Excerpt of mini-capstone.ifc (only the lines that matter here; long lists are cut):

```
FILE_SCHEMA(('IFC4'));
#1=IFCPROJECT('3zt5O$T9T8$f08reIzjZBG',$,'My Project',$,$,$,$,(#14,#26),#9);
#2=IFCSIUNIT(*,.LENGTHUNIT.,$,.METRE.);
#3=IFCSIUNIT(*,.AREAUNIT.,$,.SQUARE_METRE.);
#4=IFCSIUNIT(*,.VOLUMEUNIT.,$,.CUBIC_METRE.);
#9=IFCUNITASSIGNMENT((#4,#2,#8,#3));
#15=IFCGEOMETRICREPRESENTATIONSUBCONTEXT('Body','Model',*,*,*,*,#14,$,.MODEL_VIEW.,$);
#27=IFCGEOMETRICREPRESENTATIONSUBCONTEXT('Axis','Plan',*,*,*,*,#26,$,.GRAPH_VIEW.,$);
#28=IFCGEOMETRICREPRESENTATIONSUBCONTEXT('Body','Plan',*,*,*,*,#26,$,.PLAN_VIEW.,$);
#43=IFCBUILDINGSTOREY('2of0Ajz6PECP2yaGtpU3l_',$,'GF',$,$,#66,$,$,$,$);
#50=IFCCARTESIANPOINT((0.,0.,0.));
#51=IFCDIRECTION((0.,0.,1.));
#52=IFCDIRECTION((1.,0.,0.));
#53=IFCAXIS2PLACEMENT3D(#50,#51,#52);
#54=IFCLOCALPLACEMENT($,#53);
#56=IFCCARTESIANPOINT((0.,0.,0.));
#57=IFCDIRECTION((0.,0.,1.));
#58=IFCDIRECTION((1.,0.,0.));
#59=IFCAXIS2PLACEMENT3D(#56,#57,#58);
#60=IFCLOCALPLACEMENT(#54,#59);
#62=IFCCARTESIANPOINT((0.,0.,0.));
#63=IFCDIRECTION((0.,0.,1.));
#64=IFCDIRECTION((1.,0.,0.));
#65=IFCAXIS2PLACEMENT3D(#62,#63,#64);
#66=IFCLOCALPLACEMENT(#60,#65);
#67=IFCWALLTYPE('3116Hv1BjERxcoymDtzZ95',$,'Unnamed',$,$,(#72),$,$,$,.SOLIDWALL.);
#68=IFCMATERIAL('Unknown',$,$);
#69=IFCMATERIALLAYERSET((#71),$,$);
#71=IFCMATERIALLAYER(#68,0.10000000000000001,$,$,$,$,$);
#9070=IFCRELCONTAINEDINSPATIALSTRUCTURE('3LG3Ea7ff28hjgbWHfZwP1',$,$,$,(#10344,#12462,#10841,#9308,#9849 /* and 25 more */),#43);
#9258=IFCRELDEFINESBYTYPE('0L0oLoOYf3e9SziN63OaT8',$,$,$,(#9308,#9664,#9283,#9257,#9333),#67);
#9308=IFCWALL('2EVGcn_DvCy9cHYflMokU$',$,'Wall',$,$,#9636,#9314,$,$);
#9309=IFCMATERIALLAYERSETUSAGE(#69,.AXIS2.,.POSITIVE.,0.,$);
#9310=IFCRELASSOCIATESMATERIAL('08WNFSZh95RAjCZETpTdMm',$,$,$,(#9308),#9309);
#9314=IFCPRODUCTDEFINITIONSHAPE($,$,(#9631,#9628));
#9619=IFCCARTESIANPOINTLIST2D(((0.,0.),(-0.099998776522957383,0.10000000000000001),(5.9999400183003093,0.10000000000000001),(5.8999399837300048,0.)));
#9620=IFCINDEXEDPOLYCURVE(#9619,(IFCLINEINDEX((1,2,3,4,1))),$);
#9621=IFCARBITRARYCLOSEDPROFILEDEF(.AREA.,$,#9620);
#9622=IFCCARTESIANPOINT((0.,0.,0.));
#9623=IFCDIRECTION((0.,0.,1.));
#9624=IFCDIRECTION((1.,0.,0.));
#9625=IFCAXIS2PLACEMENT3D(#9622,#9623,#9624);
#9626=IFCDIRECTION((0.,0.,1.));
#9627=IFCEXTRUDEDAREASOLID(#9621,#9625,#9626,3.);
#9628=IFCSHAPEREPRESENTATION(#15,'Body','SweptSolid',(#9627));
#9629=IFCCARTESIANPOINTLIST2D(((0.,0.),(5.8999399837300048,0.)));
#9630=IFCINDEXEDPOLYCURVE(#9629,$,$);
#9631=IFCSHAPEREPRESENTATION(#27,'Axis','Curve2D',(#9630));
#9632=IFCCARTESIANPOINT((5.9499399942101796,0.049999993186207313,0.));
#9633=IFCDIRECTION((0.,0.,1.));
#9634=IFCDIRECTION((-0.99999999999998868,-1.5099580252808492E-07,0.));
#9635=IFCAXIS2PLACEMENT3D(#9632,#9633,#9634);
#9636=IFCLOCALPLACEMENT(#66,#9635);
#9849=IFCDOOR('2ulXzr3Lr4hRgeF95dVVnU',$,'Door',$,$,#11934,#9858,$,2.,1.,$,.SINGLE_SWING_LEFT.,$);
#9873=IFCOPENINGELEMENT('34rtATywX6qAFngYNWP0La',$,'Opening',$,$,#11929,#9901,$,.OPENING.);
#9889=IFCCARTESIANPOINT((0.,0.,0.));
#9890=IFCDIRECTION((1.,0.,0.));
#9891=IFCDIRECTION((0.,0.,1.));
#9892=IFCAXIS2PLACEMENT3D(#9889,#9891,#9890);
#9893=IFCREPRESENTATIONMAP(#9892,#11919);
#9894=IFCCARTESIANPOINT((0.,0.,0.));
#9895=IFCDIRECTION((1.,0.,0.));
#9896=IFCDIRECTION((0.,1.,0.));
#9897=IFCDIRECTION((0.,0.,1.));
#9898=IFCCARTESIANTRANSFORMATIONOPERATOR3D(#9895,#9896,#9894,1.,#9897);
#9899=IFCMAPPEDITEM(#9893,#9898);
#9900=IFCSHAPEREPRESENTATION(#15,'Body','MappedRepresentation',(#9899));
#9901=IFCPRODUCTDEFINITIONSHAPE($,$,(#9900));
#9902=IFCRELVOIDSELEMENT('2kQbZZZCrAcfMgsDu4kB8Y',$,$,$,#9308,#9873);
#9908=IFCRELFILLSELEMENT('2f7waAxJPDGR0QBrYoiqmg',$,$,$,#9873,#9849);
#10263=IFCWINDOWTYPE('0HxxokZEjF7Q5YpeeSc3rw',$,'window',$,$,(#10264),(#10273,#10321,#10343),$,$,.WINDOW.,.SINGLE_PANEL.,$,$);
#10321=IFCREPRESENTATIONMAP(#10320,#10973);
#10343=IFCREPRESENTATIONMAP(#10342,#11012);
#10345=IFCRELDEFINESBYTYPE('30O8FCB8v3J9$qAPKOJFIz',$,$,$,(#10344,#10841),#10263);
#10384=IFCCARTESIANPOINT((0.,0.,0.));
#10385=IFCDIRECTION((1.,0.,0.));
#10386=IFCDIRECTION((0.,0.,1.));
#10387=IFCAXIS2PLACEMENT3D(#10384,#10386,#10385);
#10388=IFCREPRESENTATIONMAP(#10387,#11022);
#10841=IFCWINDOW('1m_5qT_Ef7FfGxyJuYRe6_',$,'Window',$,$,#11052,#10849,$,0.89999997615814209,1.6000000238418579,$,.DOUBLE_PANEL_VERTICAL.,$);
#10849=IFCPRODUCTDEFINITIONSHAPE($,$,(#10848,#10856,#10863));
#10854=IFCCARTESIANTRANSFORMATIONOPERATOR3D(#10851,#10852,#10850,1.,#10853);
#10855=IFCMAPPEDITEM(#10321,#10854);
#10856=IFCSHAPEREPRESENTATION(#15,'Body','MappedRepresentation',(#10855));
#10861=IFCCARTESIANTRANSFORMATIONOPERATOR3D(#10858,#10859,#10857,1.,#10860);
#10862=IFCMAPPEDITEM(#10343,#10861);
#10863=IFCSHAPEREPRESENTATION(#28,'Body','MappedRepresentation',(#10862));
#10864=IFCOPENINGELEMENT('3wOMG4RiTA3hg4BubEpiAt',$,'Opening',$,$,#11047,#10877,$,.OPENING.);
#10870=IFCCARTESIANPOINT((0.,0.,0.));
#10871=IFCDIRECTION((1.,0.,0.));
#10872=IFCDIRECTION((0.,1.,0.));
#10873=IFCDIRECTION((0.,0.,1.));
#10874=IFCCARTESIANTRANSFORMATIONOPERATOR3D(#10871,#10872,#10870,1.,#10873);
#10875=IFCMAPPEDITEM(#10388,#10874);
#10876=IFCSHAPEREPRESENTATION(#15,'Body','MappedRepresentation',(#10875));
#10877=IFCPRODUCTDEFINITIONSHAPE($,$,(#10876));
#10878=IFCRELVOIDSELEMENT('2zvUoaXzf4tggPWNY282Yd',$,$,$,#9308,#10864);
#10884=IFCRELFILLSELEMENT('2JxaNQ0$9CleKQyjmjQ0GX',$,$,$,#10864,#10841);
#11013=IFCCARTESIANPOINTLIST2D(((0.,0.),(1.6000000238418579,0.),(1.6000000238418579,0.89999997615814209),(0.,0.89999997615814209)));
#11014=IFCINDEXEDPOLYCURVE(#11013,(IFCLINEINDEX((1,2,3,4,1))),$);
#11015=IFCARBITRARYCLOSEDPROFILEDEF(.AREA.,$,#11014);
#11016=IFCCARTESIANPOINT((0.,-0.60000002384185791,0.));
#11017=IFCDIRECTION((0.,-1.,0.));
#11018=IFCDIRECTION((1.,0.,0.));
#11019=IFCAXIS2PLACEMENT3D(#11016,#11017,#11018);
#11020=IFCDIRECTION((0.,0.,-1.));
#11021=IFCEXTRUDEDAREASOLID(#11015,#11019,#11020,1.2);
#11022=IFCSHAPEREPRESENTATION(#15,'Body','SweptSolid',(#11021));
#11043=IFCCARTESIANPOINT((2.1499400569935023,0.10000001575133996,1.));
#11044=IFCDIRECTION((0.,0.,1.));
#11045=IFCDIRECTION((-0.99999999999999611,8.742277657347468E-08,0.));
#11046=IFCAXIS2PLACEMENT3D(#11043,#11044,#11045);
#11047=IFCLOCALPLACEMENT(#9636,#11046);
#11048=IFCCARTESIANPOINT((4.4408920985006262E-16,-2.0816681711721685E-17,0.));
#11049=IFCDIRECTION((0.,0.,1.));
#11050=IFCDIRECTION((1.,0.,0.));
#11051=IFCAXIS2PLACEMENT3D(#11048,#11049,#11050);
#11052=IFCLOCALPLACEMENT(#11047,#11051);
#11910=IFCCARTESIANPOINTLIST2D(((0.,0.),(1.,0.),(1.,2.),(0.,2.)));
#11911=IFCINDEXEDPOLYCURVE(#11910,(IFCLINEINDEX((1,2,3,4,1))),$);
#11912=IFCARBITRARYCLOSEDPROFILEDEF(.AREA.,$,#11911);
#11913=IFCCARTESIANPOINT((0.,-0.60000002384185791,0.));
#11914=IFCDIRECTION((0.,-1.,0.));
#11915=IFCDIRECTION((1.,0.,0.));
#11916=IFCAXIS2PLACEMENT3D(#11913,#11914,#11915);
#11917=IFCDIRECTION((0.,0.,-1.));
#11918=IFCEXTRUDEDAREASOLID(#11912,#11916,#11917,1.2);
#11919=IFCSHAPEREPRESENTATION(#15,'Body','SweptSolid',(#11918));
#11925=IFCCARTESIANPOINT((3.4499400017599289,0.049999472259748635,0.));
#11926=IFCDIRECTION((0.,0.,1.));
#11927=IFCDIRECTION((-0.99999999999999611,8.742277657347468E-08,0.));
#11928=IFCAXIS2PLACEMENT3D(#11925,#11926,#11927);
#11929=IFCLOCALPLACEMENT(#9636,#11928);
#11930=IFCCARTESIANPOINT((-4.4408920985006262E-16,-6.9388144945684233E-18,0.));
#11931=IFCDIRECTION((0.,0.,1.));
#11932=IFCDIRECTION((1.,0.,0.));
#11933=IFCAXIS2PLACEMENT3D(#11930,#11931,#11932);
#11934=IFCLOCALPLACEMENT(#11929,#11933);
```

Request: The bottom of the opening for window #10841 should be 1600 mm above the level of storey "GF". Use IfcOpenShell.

```python
import numpy as np
import ifcopenshell
import ifcopenshell.api.geometry
import ifcopenshell.geom
import ifcopenshell.util.element
import ifcopenshell.util.placement
import ifcopenshell.util.shape
import ifcopenshell.util.unit

model = ifcopenshell.open("mini-capstone.ifc")
unit_scale = ifcopenshell.util.unit.calculate_unit_scale(model)

window = model.by_guid("1m_5qT_Ef7FfGxyJuYRe6_")
opening = window.FillsVoids[0].RelatingOpeningElement
storey = ifcopenshell.util.element.get_container(window, ifc_class="IfcBuildingStorey")
level = ifcopenshell.util.placement.get_local_placement(storey.ObjectPlacement)[2, 3]

# The opening's origin need not be at the sill, so measure its lowest point.
shape = ifcopenshell.geom.create_shape(ifcopenshell.geom.settings(), opening)
bottom = ifcopenshell.util.shape.get_shape_bottom_elevation(shape, shape.geometry) / unit_scale
dz = level + 1.6 / unit_scale - bottom

shift = np.array([0.0, 0.0, dz])
# The window is placed relative to its opening, so it follows when the opening moves.
matrix = ifcopenshell.util.placement.get_local_placement(opening.ObjectPlacement)
matrix[:3, 3] += shift
ifcopenshell.api.geometry.edit_object_placement(
    model, product=opening, matrix=matrix, is_si=False, should_transform_children=True
)

print(f"moved by {dz * unit_scale:+.3f} m")

model.write("mini-capstone-out.ifc")
```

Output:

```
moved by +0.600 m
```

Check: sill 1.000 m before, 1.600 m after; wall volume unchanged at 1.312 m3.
